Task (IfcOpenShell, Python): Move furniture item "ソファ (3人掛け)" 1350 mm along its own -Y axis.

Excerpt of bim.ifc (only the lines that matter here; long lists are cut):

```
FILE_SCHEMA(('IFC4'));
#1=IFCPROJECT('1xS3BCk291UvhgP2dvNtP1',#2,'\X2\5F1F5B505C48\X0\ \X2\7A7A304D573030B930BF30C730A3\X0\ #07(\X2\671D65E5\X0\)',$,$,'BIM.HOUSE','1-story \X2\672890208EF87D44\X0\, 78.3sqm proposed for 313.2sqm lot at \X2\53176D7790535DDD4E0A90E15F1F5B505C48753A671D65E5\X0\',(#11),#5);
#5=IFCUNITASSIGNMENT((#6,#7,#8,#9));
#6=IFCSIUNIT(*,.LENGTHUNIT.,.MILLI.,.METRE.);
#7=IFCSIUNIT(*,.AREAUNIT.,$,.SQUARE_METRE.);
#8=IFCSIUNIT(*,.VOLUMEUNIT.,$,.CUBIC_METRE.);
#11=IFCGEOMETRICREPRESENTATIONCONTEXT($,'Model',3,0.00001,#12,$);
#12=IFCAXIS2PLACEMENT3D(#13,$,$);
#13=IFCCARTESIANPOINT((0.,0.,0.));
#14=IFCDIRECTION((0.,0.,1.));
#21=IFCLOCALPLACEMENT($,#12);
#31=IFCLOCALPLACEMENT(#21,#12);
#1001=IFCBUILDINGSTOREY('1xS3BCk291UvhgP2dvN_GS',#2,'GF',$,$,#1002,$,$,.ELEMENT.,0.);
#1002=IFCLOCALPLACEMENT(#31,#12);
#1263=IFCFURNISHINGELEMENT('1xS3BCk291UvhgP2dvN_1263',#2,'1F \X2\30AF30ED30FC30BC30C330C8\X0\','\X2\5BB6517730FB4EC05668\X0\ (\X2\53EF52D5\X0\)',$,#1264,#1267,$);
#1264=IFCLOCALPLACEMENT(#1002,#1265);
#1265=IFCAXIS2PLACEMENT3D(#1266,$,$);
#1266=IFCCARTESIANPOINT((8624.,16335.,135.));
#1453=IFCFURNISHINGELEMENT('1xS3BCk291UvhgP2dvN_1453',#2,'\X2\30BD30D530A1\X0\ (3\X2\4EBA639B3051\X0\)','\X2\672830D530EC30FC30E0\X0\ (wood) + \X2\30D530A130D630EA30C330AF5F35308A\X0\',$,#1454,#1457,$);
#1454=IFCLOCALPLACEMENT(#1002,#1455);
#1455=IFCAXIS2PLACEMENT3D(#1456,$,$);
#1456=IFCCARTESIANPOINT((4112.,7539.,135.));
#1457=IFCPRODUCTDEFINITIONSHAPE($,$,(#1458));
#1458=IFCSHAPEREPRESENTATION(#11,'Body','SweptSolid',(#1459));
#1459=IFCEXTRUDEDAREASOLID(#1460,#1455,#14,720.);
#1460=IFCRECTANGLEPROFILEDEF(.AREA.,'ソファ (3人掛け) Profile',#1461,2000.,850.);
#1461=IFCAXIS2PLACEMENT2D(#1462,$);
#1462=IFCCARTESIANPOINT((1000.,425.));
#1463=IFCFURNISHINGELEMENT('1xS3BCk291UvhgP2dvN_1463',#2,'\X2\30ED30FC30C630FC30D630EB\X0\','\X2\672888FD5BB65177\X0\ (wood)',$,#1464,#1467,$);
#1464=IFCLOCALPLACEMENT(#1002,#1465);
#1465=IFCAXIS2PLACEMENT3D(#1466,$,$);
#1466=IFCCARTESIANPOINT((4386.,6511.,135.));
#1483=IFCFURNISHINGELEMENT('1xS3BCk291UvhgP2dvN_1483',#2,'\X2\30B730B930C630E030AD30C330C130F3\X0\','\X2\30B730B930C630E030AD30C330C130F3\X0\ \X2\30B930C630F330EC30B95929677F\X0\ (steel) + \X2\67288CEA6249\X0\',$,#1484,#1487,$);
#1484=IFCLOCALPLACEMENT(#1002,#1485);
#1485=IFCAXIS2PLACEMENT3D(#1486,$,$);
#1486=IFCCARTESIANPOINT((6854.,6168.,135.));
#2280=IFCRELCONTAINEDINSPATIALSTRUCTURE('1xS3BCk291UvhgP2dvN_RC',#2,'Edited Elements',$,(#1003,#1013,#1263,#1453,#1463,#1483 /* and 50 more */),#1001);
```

```python
import ifcopenshell
import ifcopenshell.api.geometry
import ifcopenshell.util.placement
import ifcopenshell.util.unit

model = ifcopenshell.open("bim.ifc")
unit_scale = ifcopenshell.util.unit.calculate_unit_scale(model)

item = model.by_id(1453)
matrix = ifcopenshell.util.placement.get_local_placement(item.ObjectPlacement)
matrix[:3, 3] -= matrix[:3, 1] * 1.35 / unit_scale
ifcopenshell.api.geometry.edit_object_placement(model, product=item, matrix=matrix, is_si=False)

print(ifcopenshell.util.placement.get_local_placement(item.ObjectPlacement).round(3) + 0.0)

model.write("bim_edited.ifc")
```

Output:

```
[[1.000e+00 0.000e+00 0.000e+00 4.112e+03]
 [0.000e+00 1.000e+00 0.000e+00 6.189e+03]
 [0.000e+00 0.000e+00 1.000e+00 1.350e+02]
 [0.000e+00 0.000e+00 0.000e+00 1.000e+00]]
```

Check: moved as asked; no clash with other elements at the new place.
